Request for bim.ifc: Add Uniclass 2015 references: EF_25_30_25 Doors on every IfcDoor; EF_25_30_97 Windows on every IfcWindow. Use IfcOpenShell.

First a look at what the model holds.

```python
import ifcopenshell

model = ifcopenshell.open("bim.ifc")
print(model.schema)
print("classifications:", [c.Name for c in model.by_type("IfcClassification")])
for ifc_class in ("IfcDoor", "IfcRoof", "IfcStair", "IfcWall", "IfcWindow"):
    print(ifc_class, len(model.by_type(ifc_class)))
```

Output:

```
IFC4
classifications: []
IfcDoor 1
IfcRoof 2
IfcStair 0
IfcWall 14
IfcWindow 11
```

```python
import ifcopenshell
import ifcopenshell.api.classification

model = ifcopenshell.open("bim.ifc")

system = ifcopenshell.api.classification.add_classification(model, classification="Uniclass 2015")

codes = {
    "IfcDoor": ("EF_25_30_25", "Doors"),
    "IfcWindow": ("EF_25_30_97", "Windows"),
}
for ifc_class, (code, name) in codes.items():
    products = model.by_type(ifc_class)
    ifcopenshell.api.classification.add_reference(
        model, products=products, classification=system, identification=code, name=name
    )
    print(code, len(products))

model.write("bim_edited.ifc")
```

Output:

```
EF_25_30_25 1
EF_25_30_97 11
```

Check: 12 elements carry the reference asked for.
